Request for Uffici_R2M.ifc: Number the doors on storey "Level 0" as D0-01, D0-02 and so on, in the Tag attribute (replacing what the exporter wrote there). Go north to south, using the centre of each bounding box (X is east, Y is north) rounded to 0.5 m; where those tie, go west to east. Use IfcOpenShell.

First a look at what the model holds.

```python
import ifcopenshell
import ifcopenshell.util.element
import ifcopenshell.util.placement

model = ifcopenshell.open("Uffici_R2M.ifc")
print(model.schema)
storey = next(s for s in model.by_type("IfcBuildingStorey") if s.Name == "Level 0")
doors = [e for e in ifcopenshell.util.element.get_decomposition(storey) if e.is_a("IfcDoor")]
for e in sorted(doors, key=lambda e: e.id()):
    origin = ifcopenshell.util.placement.get_local_placement(e.ObjectPlacement)[:3, 3]
    print(e.id(), e.Tag, e.Name, origin.round(2) + 0.0, sep=" | ")
```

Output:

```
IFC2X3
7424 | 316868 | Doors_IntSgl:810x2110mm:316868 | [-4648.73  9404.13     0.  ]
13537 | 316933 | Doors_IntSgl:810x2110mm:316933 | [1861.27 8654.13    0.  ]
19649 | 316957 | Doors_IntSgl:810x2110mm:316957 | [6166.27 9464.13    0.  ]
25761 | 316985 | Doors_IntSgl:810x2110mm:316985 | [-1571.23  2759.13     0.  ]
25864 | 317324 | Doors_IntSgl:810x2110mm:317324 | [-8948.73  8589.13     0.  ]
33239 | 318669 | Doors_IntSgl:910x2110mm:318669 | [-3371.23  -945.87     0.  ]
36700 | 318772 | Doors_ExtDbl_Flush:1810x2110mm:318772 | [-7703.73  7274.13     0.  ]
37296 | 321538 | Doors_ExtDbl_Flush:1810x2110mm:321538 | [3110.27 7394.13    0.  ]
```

```python
import ifcopenshell
import ifcopenshell.geom
import ifcopenshell.util.element
import ifcopenshell.util.shape

model = ifcopenshell.open("Uffici_R2M.ifc")
settings = ifcopenshell.geom.settings()
settings.set("use-world-coords", True)


def centre(element):
    shape = ifcopenshell.geom.create_shape(settings, element)
    return ifcopenshell.util.shape.get_bbox_centroid(shape.geometry)


storey = next(s for s in model.by_type("IfcBuildingStorey") if s.Name == "Level 0")
doors = [e for e in ifcopenshell.util.element.get_decomposition(storey) if e.is_a("IfcDoor")]

# Insertion points can sit at a corner or the storey origin, so sort by the geometry (in metres).
centres = {e: centre(e) for e in doors}
doors.sort(key=lambda e: (-round(centres[e][1] / 0.5), centres[e][0]))

for i, e in enumerate(doors, start=1):
    number = f"D0-{i:02d}"
    e.Tag = number
    print(e.id(), number)

model.write("Uffici_R2M_edited.ifc")
```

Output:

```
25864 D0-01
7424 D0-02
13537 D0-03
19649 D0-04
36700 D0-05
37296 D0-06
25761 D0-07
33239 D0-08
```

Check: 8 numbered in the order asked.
